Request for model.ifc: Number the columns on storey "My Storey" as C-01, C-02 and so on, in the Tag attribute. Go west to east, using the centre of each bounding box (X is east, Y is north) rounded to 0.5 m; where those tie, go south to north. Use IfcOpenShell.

First a look at what the model holds.

```python
import ifcopenshell
import ifcopenshell.util.element
import ifcopenshell.util.placement

model = ifcopenshell.open("model.ifc")
print(model.schema)
storey = next(s for s in model.by_type("IfcBuildingStorey") if s.Name == "My Storey")
columns = [e for e in ifcopenshell.util.element.get_decomposition(storey) if e.is_a("IfcColumn")]
for e in sorted(columns, key=lambda e: e.id()):
    origin = ifcopenshell.util.placement.get_local_placement(e.ObjectPlacement)[:3, 3]
    print(e.id(), e.Tag, e.Name, origin.round(2) + 0.0, sep=" | ")
```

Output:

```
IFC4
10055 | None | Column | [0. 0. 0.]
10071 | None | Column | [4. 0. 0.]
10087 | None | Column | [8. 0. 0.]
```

```python
import ifcopenshell
import ifcopenshell.geom
import ifcopenshell.util.element
import ifcopenshell.util.shape

model = ifcopenshell.open("model.ifc")
settings = ifcopenshell.geom.settings()
settings.set("use-world-coords", True)


def centre(element):
    shape = ifcopenshell.geom.create_shape(settings, element)
    return ifcopenshell.util.shape.get_bbox_centroid(shape.geometry)


storey = next(s for s in model.by_type("IfcBuildingStorey") if s.Name == "My Storey")
columns = [e for e in ifcopenshell.util.element.get_decomposition(storey) if e.is_a("IfcColumn")]

# Insertion points can sit at a corner or the storey origin, so sort by the geometry (in metres).
centres = {e: centre(e) for e in columns}
columns.sort(key=lambda e: (round(centres[e][0] / 0.5), centres[e][1]))

for i, e in enumerate(columns, start=1):
    number = f"C-{i:02d}"
    e.Tag = number
    print(e.id(), number)

model.write("model_rev.ifc")
```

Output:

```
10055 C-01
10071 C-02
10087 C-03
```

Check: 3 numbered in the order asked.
